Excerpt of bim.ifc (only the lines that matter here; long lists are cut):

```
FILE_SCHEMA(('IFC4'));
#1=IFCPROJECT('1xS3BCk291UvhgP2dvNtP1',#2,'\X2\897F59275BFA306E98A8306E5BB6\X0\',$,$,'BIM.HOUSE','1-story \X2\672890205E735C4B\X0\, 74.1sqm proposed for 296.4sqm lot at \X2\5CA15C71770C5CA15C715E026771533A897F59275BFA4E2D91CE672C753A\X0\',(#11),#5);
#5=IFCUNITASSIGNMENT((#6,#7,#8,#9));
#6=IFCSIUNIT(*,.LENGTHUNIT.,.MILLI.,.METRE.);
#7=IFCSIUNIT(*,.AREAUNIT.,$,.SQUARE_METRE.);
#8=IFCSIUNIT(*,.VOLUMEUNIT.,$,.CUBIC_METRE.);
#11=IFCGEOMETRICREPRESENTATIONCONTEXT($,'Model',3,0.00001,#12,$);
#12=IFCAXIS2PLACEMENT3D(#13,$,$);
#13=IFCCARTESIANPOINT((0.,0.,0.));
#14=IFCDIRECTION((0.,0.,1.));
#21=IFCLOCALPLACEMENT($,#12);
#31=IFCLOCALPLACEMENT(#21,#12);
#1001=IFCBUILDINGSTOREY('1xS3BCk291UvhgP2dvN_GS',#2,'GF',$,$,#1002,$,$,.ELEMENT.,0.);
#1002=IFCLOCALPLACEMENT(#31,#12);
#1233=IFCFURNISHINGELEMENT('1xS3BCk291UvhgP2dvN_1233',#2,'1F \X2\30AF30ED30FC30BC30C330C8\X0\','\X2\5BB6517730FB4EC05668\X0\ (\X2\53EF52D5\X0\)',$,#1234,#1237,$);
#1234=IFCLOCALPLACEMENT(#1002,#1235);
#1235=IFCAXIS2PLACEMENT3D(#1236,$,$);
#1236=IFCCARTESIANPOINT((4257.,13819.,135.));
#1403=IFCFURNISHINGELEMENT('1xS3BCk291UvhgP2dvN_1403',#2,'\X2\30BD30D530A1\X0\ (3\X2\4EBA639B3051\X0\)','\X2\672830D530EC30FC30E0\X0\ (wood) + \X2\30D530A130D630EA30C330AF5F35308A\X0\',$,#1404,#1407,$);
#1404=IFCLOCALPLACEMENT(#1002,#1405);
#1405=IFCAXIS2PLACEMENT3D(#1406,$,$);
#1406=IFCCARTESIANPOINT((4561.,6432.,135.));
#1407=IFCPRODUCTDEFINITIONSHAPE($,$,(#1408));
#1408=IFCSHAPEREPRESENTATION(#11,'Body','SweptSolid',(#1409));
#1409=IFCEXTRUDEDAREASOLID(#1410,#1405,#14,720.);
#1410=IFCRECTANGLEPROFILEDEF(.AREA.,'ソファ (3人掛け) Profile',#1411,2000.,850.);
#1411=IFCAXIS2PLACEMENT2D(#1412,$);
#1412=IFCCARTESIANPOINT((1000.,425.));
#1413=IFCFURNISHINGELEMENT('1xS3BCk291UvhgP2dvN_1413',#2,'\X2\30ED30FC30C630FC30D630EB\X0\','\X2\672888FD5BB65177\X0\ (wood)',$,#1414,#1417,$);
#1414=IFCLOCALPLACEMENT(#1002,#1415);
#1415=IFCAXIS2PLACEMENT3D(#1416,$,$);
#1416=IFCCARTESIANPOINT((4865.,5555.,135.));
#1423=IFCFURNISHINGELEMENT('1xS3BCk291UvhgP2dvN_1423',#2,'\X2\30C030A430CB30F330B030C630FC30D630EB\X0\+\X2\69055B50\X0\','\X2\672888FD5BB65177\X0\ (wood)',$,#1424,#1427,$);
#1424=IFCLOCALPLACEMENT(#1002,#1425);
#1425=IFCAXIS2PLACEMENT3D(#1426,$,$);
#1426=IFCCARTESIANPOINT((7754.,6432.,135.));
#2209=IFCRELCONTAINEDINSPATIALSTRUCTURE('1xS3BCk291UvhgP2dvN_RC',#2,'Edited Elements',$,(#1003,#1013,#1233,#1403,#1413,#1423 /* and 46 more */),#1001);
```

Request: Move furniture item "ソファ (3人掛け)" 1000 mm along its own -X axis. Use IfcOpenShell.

```python
import ifcopenshell
import ifcopenshell.api.geometry
import ifcopenshell.util.placement
import ifcopenshell.util.unit

model = ifcopenshell.open("bim.ifc")
unit_scale = ifcopenshell.util.unit.calculate_unit_scale(model)

item = model.by_id(1403)
matrix = ifcopenshell.util.placement.get_local_placement(item.ObjectPlacement)
matrix[:3, 3] -= matrix[:3, 0] * 1 / unit_scale
ifcopenshell.api.geometry.edit_object_placement(model, product=item, matrix=matrix, is_si=False)

print(ifcopenshell.util.placement.get_local_placement(item.ObjectPlacement).round(3) + 0.0)

model.write("bim_rev.ifc")
```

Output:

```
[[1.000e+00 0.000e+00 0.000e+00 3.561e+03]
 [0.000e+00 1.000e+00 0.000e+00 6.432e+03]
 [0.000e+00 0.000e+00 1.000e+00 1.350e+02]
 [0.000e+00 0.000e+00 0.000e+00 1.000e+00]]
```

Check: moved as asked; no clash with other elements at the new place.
